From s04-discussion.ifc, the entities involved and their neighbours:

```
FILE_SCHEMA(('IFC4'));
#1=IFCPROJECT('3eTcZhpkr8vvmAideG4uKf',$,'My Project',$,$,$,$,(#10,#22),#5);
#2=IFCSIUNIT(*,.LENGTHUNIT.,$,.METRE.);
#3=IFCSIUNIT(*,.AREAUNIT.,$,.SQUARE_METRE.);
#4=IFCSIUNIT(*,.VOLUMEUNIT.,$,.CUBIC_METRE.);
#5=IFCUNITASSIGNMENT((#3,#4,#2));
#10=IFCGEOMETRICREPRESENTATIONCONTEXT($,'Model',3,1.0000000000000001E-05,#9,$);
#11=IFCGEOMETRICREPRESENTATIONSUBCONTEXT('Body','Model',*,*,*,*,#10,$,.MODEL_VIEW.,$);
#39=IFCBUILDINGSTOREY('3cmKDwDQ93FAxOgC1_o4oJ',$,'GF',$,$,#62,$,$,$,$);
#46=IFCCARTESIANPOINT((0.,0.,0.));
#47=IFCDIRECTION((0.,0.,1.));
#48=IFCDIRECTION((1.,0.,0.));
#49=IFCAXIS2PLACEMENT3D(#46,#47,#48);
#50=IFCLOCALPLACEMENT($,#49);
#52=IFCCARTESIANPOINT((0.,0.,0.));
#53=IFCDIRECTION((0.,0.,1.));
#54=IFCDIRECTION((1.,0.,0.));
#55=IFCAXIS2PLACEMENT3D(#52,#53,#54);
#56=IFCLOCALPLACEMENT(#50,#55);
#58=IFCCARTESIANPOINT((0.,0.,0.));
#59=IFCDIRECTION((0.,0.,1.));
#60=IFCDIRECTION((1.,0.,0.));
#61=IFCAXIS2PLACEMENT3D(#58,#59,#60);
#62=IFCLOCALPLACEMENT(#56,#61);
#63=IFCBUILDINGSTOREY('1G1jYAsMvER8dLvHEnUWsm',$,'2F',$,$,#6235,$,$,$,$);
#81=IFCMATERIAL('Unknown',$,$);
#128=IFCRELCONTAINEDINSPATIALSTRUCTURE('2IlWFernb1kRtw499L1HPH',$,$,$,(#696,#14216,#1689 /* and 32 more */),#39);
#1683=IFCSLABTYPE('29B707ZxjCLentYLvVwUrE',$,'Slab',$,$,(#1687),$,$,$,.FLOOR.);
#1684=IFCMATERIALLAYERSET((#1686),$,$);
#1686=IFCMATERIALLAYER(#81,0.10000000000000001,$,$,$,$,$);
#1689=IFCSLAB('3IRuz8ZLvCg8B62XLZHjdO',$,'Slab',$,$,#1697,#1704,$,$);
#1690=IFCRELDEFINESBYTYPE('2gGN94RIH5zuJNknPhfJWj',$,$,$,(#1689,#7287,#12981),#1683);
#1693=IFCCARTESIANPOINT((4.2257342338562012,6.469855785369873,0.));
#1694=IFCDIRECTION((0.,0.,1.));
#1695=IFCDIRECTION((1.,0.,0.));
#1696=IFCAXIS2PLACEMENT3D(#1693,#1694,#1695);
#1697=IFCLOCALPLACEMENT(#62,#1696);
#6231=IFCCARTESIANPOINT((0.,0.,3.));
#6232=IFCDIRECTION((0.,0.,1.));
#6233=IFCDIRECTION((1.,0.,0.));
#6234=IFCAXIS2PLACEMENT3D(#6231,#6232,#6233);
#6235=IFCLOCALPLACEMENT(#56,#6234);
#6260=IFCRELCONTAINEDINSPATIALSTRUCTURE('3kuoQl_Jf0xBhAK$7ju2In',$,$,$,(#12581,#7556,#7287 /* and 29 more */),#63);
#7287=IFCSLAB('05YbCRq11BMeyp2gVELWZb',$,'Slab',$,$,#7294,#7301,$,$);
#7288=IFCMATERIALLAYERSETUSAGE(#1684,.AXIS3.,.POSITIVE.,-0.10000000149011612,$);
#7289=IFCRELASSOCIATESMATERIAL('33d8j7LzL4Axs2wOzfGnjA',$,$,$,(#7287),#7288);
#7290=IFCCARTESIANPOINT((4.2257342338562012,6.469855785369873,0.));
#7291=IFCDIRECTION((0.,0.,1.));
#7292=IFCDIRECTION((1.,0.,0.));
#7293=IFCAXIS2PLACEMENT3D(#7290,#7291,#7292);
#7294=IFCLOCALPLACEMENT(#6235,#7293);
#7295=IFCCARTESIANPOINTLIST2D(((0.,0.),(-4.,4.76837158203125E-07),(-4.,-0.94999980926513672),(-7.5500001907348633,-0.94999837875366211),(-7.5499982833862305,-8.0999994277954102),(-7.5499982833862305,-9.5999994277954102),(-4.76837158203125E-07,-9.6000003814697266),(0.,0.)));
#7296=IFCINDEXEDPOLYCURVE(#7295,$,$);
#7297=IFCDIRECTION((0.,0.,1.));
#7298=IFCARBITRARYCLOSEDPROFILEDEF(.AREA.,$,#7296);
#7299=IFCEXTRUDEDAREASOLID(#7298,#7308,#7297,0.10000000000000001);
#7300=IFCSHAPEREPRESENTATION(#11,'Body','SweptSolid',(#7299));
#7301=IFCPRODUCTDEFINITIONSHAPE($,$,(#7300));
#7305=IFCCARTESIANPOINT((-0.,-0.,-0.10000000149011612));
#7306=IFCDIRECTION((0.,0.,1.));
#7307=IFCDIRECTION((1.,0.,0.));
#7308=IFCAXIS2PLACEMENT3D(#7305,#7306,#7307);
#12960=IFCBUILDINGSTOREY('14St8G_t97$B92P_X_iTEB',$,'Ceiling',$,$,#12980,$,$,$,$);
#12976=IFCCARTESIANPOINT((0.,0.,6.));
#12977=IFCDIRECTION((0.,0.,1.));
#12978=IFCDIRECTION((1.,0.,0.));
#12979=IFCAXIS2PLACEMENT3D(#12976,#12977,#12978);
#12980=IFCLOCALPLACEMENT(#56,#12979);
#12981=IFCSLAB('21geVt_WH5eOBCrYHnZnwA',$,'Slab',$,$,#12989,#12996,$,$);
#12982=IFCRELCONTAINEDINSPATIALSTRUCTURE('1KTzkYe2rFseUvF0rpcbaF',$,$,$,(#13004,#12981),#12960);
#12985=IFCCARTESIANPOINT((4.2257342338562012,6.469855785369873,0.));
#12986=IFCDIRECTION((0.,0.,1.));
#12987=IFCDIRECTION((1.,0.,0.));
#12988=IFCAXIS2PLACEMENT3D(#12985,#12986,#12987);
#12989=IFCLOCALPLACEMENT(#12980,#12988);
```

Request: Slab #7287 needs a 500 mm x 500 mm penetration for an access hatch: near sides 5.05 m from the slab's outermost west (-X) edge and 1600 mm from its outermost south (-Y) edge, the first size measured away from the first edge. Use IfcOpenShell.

```python
import numpy as np
import ifcopenshell
import ifcopenshell.api.feature
import ifcopenshell.api.geometry
import ifcopenshell.api.root
import ifcopenshell.geom
import ifcopenshell.util.placement
import ifcopenshell.util.representation
import ifcopenshell.util.shape
import ifcopenshell.util.unit

model = ifcopenshell.open("s04-discussion.ifc")
unit_scale = ifcopenshell.util.unit.calculate_unit_scale(model)
settings = ifcopenshell.geom.settings()


def volume(element):
    """Net volume in cubic metres, openings subtracted."""
    shape = ifcopenshell.geom.create_shape(settings, element)
    return ifcopenshell.util.shape.get_volume(shape.geometry)


slab = model.by_guid("05YbCRq11BMeyp2gVELWZb")
before = volume(slab)

# Extent in the slab's own axes, in metres. The edges named are its -X and -Y sides.
slab_shape = ifcopenshell.geom.create_shape(settings, slab)
vertices = ifcopenshell.util.shape.get_vertices(slab_shape.geometry)
x_min, y_min, bottom = vertices.min(axis=0)
top = vertices[:, 2].max()

opening = ifcopenshell.api.root.create_entity(model, ifc_class="IfcOpeningElement", name="Access hatch opening", predefined_type="OPENING")
context = ifcopenshell.util.representation.get_context(model, "Model", "Body", "MODEL_VIEW")
width, depth = 0.5, 0.5
outline = [(0.0, 0.0), (width, 0.0), (width, depth), (0.0, depth), (0.0, 0.0)]
# Overshoot both faces by 50 mm so the cut is clean.
shape = ifcopenshell.api.geometry.add_slab_representation(
    model, context=context, depth=top - bottom + 0.1, polyline=outline
)
ifcopenshell.api.geometry.assign_representation(model, product=opening, representation=shape)

matrix = ifcopenshell.util.placement.get_local_placement(slab.ObjectPlacement)
matrix[:, 3] = matrix @ np.append(np.array([x_min + 5.05, y_min + 1.6, bottom - 0.05]) / unit_scale, 1.0)
ifcopenshell.api.geometry.edit_object_placement(model, product=opening, matrix=matrix, is_si=False)
ifcopenshell.api.feature.add_feature(model, feature=opening, element=slab)

after = volume(slab)

print(f"slab volume {before:.3f} -> {after:.3f} m3")

model.write("s04-discussion_updated.ifc")
```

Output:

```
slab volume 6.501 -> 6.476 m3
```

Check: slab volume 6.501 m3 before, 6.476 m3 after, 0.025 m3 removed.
